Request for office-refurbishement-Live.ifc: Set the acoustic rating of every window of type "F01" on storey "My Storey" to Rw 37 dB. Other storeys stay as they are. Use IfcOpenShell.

First a look at what the model holds.

```python
import ifcopenshell
import ifcopenshell.util.element

model = ifcopenshell.open("office-refurbishement-Live.ifc")
print(model.schema)
storey = next(s for s in model.by_type("IfcBuildingStorey") if s.Name == "My Storey")
windows = [e for e in ifcopenshell.util.element.get_decomposition(storey) if e.is_a("IfcWindow")]
seen = {}
for e in windows:
    element_type = ifcopenshell.util.element.get_type(e)
    key = (element_type.Name if element_type != e and element_type else None, ifcopenshell.util.element.get_pset(e, "Pset_WindowCommon", "AcousticRating"))
    seen[key] = seen.get(key, 0) + 1
for (name, value), count in sorted(seen.items(), key=str):
    print(count, "x", name, "|", value)
```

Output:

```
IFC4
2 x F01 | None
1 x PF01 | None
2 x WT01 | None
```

```python
import ifcopenshell
import ifcopenshell.api.pset
import ifcopenshell.util.element

model = ifcopenshell.open("office-refurbishement-Live.ifc")

storey = next(s for s in model.by_type("IfcBuildingStorey") if s.Name == "My Storey")
windows = [e for e in ifcopenshell.util.element.get_decomposition(storey) if e.is_a("IfcWindow")]

count = 0
for e in windows:
    element_type = ifcopenshell.util.element.get_type(e)
    if element_type in (None, e) or element_type.Name != "F01":
        continue
    # add_pset returns the element's existing set when there is one.
    pset = ifcopenshell.api.pset.add_pset(model, product=e, name="Pset_WindowCommon")
    ifcopenshell.api.pset.edit_pset(model, pset=pset, properties={"AcousticRating": "Rw 37 dB"})
    count += 1

print(count, "windows updated")

model.write("office-refurbishement-Live_rev.ifc")
```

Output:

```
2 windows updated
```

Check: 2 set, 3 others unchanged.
